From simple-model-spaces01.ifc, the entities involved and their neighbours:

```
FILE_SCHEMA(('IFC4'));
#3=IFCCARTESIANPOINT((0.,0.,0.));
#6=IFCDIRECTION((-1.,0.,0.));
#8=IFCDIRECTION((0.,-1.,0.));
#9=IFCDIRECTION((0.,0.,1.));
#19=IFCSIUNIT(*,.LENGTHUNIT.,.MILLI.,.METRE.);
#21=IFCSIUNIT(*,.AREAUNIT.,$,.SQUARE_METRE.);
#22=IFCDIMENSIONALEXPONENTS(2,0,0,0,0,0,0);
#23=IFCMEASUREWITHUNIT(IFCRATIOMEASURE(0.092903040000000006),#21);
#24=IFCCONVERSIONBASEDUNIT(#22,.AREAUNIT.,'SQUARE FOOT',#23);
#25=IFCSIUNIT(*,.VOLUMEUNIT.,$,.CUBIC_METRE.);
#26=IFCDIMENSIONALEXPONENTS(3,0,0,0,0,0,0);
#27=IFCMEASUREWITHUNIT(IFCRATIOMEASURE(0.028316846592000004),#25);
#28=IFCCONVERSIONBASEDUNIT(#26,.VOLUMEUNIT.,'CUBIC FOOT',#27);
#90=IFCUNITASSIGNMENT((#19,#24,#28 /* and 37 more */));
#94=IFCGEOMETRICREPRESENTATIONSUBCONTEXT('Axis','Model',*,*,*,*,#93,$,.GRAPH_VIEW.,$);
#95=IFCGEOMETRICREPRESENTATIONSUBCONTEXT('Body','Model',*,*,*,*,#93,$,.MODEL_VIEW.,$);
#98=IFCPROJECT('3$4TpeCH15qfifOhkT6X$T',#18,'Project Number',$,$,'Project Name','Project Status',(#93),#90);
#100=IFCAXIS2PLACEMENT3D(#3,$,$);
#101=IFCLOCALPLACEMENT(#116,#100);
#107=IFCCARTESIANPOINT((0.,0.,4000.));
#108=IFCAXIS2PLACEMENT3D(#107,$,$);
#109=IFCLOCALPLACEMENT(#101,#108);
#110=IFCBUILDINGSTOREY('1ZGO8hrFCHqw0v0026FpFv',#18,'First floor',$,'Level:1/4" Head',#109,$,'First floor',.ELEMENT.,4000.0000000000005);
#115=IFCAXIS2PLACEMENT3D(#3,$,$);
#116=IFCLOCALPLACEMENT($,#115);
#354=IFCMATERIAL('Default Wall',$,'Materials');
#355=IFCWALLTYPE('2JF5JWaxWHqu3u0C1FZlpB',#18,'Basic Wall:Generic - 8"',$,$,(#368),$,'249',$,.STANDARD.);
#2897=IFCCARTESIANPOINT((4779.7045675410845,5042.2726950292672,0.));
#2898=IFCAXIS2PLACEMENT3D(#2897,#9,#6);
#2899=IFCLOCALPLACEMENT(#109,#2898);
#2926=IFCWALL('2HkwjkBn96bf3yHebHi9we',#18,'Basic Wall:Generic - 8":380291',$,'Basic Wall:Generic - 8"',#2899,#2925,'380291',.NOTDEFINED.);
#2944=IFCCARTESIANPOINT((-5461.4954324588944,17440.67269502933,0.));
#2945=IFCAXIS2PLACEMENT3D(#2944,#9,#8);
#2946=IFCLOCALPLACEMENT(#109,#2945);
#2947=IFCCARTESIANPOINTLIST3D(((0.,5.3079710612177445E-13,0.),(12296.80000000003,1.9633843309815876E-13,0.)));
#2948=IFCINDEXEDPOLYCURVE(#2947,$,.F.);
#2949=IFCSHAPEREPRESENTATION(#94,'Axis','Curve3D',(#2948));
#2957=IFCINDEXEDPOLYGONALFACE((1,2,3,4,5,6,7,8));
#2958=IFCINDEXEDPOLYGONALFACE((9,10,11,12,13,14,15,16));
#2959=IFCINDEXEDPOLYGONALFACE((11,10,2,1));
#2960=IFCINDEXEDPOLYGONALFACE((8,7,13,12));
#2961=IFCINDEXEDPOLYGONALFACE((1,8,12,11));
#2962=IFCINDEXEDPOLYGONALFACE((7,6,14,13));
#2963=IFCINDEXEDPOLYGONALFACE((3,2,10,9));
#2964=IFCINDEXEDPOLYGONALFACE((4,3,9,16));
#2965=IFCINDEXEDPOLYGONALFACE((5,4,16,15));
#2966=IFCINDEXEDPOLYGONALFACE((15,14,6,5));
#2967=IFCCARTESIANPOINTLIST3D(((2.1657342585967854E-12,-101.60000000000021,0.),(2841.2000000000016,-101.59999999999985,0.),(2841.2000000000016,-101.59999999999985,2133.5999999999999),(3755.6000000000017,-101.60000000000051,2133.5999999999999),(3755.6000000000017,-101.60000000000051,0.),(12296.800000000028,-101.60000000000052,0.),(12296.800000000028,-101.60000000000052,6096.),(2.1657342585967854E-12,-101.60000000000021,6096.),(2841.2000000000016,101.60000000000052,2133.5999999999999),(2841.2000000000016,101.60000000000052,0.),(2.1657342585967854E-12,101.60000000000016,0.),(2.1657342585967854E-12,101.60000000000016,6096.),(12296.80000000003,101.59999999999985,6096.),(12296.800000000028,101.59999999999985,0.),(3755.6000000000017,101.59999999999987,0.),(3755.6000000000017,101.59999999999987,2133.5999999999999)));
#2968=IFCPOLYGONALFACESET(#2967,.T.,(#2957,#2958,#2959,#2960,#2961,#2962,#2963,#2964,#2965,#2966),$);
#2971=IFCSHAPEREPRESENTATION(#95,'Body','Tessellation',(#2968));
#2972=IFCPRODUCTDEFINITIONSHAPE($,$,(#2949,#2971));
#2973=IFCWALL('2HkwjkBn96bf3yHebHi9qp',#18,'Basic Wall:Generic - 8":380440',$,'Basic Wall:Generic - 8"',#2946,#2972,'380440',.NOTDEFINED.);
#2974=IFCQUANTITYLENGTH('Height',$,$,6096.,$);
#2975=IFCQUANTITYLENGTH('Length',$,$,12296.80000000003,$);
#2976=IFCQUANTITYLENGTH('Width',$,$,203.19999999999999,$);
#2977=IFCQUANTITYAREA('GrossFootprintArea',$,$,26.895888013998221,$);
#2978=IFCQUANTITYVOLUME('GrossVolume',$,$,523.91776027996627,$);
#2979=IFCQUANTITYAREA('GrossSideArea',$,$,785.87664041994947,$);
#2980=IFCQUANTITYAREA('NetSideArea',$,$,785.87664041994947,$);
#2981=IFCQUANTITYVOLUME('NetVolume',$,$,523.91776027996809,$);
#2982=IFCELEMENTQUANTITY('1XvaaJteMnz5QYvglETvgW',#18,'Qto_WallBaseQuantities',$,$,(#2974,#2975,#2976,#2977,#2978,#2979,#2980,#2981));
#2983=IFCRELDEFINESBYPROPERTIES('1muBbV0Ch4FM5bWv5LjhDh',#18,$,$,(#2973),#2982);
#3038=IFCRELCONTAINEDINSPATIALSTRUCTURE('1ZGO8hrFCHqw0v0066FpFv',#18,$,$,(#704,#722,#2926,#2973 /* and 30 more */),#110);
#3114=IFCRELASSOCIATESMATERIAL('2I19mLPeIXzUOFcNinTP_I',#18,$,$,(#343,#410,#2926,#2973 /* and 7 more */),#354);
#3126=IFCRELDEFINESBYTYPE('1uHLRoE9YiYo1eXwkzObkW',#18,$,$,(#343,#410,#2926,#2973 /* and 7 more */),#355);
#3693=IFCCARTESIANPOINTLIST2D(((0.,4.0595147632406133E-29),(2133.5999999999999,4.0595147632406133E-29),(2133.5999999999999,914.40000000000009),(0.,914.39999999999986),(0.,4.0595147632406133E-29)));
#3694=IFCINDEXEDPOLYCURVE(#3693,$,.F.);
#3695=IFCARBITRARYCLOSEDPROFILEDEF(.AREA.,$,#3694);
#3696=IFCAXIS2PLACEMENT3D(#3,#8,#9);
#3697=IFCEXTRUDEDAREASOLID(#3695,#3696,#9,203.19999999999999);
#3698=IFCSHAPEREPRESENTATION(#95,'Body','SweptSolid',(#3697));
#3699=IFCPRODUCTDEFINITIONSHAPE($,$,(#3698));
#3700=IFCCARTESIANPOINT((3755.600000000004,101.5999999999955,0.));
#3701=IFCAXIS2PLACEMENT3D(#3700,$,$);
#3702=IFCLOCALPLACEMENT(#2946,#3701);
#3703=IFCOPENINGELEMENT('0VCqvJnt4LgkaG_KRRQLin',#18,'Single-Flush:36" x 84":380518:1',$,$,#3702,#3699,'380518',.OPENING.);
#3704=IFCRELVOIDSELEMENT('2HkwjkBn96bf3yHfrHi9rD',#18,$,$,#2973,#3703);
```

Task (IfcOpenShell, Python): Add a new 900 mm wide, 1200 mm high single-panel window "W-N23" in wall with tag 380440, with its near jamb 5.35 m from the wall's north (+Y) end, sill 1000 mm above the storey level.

```python
import numpy as np
import ifcopenshell
import ifcopenshell.api.feature
import ifcopenshell.api.geometry
import ifcopenshell.api.pset
import ifcopenshell.api.root
import ifcopenshell.api.spatial
import ifcopenshell.geom
import ifcopenshell.util.element
import ifcopenshell.util.placement
import ifcopenshell.util.representation
import ifcopenshell.util.shape
import ifcopenshell.util.unit

model = ifcopenshell.open("simple-model-spaces01.ifc")
unit_scale = ifcopenshell.util.unit.calculate_unit_scale(model)
area_scale = ifcopenshell.util.unit.calculate_unit_scale(model, "AREAUNIT")
volume_scale = ifcopenshell.util.unit.calculate_unit_scale(model, "VOLUMEUNIT")
settings = ifcopenshell.geom.settings()


def volume(element):
    """Net volume in cubic metres, openings subtracted."""
    shape = ifcopenshell.geom.create_shape(settings, element)
    return ifcopenshell.util.shape.get_volume(shape.geometry)


wall = model.by_guid("2HkwjkBn96bf3yHebHi9qp")
storey = ifcopenshell.util.element.get_container(wall, ifc_class="IfcBuildingStorey")
context = ifcopenshell.util.representation.get_context(model, "Model", "Body", "MODEL_VIEW")
before = volume(wall)

width, height, from_end, sill = 0.9, 1.2, 5.35, 1  # metres

# The wall runs along its own X axis, and the end named is its -X end.
wall_shape = ifcopenshell.geom.create_shape(settings, wall)
x, y, z = ifcopenshell.util.shape.get_vertices(wall_shape.geometry).T
start = x.min() + from_end
face, thickness = float(y.min()), float(y.max() - y.min())
wall_matrix = ifcopenshell.util.placement.get_local_placement(wall.ObjectPlacement)
level = ifcopenshell.util.placement.get_local_placement(storey.ObjectPlacement)[2, 3]


def in_wall(x, y):
    """Placement at x, y metres in the wall's axes, at sill height."""
    matrix = wall_matrix.copy()
    matrix[:, 3] = wall_matrix @ np.array([x / unit_scale, y / unit_scale, 0.0, 1.0])
    matrix[2, 3] = level + sill / unit_scale
    return matrix


# Opening: a box that overshoots both wall faces by 50 mm.
opening = ifcopenshell.api.root.create_entity(model, ifc_class="IfcOpeningElement", predefined_type="OPENING")
box = ifcopenshell.api.geometry.add_wall_representation(
    model, context=context, length=width, height=height, thickness=thickness + 0.1
)
ifcopenshell.api.geometry.assign_representation(model, product=opening, representation=box)
ifcopenshell.api.geometry.edit_object_placement(model, product=opening, matrix=in_wall(start, face - 0.05), is_si=False)
ifcopenshell.api.feature.add_feature(model, feature=opening, element=wall)

window = ifcopenshell.api.root.create_entity(model, ifc_class="IfcWindow", name="W-N23", predefined_type="WINDOW")
window.OverallWidth, window.OverallHeight = width / unit_scale, height / unit_scale
window.PartitioningType = "SINGLE_PANEL"
body = ifcopenshell.api.geometry.add_window_representation(
    model,
    context=context,
    overall_width=window.OverallWidth,
    overall_height=window.OverallHeight,
    partition_type="SINGLE_PANEL",
)
ifcopenshell.api.geometry.assign_representation(model, product=window, representation=body)
ifcopenshell.api.spatial.assign_container(model, products=[window], relating_structure=storey)
ifcopenshell.api.feature.add_filling(model, opening=opening, element=window)

# Centre the window in the wall's thickness.
ifcopenshell.api.geometry.edit_object_placement(model, product=window, matrix=in_wall(start, face), is_si=False)
window_shape = ifcopenshell.geom.create_shape(settings, window)
depth = ifcopenshell.util.shape.get_vertices(window_shape.geometry)[:, 1]
offset = face + thickness / 2 - (depth.min() + depth.max()) / 2
ifcopenshell.api.geometry.edit_object_placement(model, product=window, matrix=in_wall(start, offset), is_si=False)

after = volume(wall)

# Update the wall's stored quantities.
qto = model.by_id(ifcopenshell.util.element.get_pset(wall, "Qto_WallBaseQuantities", should_inherit=False)["id"])
ifcopenshell.api.pset.edit_qto(model, qto=qto, properties={
    "NetSideArea": after / thickness / area_scale,
    "NetVolume": after / volume_scale,
})

print(f"wall volume {before:.3f} -> {after:.3f} m3")

model.write("simple-model-spaces01_updated.ifc")
```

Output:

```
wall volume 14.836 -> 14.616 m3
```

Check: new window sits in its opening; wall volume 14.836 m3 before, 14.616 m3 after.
